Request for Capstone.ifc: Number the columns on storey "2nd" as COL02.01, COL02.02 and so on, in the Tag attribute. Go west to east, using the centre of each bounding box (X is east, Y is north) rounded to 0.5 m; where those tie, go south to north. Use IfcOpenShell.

First a look at what the model holds.

```python
import ifcopenshell
import ifcopenshell.util.element
import ifcopenshell.util.placement

model = ifcopenshell.open("Capstone.ifc")
print(model.schema)
storey = next(s for s in model.by_type("IfcBuildingStorey") if s.Name == "2nd")
columns = [e for e in ifcopenshell.util.element.get_decomposition(storey) if e.is_a("IfcColumn")]
for e in sorted(columns, key=lambda e: e.id()):
    origin = ifcopenshell.util.placement.get_local_placement(e.ObjectPlacement)[:3, 3]
    print(e.id(), e.Tag, e.Name, origin.round(2) + 0.0, sep=" | ")
```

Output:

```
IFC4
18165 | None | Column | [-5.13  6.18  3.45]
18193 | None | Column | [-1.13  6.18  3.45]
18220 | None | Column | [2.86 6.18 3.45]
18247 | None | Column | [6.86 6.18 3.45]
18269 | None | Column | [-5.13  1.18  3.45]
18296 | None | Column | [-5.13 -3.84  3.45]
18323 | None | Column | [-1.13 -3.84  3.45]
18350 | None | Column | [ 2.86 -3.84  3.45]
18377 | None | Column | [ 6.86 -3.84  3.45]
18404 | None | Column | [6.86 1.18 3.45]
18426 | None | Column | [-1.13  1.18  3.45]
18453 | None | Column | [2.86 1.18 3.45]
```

```python
import ifcopenshell
import ifcopenshell.geom
import ifcopenshell.util.element
import ifcopenshell.util.shape

model = ifcopenshell.open("Capstone.ifc")
settings = ifcopenshell.geom.settings()
settings.set("use-world-coords", True)


def centre(element):
    shape = ifcopenshell.geom.create_shape(settings, element)
    return ifcopenshell.util.shape.get_bbox_centroid(shape.geometry)


storey = next(s for s in model.by_type("IfcBuildingStorey") if s.Name == "2nd")
columns = [e for e in ifcopenshell.util.element.get_decomposition(storey) if e.is_a("IfcColumn")]

# Insertion points can sit at a corner or the storey origin, so sort by the geometry (in metres).
centres = {e: centre(e) for e in columns}
columns.sort(key=lambda e: (round(centres[e][0] / 0.5), centres[e][1]))

for i, e in enumerate(columns, start=1):
    number = f"COL02.{i:02d}"
    e.Tag = number
    print(e.id(), number)

model.write("Capstone_edited.ifc")
```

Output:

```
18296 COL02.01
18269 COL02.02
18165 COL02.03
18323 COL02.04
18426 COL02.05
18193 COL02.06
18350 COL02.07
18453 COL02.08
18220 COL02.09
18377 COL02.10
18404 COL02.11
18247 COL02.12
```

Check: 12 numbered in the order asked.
